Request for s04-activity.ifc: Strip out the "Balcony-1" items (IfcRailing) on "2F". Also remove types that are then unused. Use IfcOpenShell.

First a look at what the model holds.

```python
import ifcopenshell
import ifcopenshell.util.element

model = ifcopenshell.open("s04-activity.ifc")
print(model.schema)
storey = next(s for s in model.by_type("IfcBuildingStorey") if s.Name == "2F")
railings = [e for e in ifcopenshell.util.element.get_decomposition(storey) if e.is_a("IfcRailing")]
seen = {}
for e in railings:
    element_type = ifcopenshell.util.element.get_type(e)
    name = element_type.Name if element_type not in (None, e) else None
    seen[name] = seen.get(name, 0) + 1
for name, count in sorted(seen.items(), key=str):
    print(count, "x", name)
```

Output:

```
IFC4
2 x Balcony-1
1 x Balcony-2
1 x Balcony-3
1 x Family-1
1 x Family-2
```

```python
import ifcopenshell
import ifcopenshell.api.root
import ifcopenshell.util.element

model = ifcopenshell.open("s04-activity.ifc")

storey = next(s for s in model.by_type("IfcBuildingStorey") if s.Name == "2F")
railings = [e for e in ifcopenshell.util.element.get_decomposition(storey) if e.is_a("IfcRailing")]
targets = [e for e in railings if (t := ifcopenshell.util.element.get_type(e)) not in (None, e) and t.Name == "Balcony-1"]
types = {ifcopenshell.util.element.get_type(e) for e in targets} - {None, *targets}

for e in targets:
    ifcopenshell.api.root.remove_product(model, product=e)
print(len(targets), "removed")

unused = [t for t in types if not ifcopenshell.util.element.get_types(t)]
for t in unused:
    ifcopenshell.api.root.remove_product(model, product=t)
print(len(unused), "unused types removed")

model.write("s04-activity_rev.ifc")
```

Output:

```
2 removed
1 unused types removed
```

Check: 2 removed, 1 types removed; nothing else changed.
